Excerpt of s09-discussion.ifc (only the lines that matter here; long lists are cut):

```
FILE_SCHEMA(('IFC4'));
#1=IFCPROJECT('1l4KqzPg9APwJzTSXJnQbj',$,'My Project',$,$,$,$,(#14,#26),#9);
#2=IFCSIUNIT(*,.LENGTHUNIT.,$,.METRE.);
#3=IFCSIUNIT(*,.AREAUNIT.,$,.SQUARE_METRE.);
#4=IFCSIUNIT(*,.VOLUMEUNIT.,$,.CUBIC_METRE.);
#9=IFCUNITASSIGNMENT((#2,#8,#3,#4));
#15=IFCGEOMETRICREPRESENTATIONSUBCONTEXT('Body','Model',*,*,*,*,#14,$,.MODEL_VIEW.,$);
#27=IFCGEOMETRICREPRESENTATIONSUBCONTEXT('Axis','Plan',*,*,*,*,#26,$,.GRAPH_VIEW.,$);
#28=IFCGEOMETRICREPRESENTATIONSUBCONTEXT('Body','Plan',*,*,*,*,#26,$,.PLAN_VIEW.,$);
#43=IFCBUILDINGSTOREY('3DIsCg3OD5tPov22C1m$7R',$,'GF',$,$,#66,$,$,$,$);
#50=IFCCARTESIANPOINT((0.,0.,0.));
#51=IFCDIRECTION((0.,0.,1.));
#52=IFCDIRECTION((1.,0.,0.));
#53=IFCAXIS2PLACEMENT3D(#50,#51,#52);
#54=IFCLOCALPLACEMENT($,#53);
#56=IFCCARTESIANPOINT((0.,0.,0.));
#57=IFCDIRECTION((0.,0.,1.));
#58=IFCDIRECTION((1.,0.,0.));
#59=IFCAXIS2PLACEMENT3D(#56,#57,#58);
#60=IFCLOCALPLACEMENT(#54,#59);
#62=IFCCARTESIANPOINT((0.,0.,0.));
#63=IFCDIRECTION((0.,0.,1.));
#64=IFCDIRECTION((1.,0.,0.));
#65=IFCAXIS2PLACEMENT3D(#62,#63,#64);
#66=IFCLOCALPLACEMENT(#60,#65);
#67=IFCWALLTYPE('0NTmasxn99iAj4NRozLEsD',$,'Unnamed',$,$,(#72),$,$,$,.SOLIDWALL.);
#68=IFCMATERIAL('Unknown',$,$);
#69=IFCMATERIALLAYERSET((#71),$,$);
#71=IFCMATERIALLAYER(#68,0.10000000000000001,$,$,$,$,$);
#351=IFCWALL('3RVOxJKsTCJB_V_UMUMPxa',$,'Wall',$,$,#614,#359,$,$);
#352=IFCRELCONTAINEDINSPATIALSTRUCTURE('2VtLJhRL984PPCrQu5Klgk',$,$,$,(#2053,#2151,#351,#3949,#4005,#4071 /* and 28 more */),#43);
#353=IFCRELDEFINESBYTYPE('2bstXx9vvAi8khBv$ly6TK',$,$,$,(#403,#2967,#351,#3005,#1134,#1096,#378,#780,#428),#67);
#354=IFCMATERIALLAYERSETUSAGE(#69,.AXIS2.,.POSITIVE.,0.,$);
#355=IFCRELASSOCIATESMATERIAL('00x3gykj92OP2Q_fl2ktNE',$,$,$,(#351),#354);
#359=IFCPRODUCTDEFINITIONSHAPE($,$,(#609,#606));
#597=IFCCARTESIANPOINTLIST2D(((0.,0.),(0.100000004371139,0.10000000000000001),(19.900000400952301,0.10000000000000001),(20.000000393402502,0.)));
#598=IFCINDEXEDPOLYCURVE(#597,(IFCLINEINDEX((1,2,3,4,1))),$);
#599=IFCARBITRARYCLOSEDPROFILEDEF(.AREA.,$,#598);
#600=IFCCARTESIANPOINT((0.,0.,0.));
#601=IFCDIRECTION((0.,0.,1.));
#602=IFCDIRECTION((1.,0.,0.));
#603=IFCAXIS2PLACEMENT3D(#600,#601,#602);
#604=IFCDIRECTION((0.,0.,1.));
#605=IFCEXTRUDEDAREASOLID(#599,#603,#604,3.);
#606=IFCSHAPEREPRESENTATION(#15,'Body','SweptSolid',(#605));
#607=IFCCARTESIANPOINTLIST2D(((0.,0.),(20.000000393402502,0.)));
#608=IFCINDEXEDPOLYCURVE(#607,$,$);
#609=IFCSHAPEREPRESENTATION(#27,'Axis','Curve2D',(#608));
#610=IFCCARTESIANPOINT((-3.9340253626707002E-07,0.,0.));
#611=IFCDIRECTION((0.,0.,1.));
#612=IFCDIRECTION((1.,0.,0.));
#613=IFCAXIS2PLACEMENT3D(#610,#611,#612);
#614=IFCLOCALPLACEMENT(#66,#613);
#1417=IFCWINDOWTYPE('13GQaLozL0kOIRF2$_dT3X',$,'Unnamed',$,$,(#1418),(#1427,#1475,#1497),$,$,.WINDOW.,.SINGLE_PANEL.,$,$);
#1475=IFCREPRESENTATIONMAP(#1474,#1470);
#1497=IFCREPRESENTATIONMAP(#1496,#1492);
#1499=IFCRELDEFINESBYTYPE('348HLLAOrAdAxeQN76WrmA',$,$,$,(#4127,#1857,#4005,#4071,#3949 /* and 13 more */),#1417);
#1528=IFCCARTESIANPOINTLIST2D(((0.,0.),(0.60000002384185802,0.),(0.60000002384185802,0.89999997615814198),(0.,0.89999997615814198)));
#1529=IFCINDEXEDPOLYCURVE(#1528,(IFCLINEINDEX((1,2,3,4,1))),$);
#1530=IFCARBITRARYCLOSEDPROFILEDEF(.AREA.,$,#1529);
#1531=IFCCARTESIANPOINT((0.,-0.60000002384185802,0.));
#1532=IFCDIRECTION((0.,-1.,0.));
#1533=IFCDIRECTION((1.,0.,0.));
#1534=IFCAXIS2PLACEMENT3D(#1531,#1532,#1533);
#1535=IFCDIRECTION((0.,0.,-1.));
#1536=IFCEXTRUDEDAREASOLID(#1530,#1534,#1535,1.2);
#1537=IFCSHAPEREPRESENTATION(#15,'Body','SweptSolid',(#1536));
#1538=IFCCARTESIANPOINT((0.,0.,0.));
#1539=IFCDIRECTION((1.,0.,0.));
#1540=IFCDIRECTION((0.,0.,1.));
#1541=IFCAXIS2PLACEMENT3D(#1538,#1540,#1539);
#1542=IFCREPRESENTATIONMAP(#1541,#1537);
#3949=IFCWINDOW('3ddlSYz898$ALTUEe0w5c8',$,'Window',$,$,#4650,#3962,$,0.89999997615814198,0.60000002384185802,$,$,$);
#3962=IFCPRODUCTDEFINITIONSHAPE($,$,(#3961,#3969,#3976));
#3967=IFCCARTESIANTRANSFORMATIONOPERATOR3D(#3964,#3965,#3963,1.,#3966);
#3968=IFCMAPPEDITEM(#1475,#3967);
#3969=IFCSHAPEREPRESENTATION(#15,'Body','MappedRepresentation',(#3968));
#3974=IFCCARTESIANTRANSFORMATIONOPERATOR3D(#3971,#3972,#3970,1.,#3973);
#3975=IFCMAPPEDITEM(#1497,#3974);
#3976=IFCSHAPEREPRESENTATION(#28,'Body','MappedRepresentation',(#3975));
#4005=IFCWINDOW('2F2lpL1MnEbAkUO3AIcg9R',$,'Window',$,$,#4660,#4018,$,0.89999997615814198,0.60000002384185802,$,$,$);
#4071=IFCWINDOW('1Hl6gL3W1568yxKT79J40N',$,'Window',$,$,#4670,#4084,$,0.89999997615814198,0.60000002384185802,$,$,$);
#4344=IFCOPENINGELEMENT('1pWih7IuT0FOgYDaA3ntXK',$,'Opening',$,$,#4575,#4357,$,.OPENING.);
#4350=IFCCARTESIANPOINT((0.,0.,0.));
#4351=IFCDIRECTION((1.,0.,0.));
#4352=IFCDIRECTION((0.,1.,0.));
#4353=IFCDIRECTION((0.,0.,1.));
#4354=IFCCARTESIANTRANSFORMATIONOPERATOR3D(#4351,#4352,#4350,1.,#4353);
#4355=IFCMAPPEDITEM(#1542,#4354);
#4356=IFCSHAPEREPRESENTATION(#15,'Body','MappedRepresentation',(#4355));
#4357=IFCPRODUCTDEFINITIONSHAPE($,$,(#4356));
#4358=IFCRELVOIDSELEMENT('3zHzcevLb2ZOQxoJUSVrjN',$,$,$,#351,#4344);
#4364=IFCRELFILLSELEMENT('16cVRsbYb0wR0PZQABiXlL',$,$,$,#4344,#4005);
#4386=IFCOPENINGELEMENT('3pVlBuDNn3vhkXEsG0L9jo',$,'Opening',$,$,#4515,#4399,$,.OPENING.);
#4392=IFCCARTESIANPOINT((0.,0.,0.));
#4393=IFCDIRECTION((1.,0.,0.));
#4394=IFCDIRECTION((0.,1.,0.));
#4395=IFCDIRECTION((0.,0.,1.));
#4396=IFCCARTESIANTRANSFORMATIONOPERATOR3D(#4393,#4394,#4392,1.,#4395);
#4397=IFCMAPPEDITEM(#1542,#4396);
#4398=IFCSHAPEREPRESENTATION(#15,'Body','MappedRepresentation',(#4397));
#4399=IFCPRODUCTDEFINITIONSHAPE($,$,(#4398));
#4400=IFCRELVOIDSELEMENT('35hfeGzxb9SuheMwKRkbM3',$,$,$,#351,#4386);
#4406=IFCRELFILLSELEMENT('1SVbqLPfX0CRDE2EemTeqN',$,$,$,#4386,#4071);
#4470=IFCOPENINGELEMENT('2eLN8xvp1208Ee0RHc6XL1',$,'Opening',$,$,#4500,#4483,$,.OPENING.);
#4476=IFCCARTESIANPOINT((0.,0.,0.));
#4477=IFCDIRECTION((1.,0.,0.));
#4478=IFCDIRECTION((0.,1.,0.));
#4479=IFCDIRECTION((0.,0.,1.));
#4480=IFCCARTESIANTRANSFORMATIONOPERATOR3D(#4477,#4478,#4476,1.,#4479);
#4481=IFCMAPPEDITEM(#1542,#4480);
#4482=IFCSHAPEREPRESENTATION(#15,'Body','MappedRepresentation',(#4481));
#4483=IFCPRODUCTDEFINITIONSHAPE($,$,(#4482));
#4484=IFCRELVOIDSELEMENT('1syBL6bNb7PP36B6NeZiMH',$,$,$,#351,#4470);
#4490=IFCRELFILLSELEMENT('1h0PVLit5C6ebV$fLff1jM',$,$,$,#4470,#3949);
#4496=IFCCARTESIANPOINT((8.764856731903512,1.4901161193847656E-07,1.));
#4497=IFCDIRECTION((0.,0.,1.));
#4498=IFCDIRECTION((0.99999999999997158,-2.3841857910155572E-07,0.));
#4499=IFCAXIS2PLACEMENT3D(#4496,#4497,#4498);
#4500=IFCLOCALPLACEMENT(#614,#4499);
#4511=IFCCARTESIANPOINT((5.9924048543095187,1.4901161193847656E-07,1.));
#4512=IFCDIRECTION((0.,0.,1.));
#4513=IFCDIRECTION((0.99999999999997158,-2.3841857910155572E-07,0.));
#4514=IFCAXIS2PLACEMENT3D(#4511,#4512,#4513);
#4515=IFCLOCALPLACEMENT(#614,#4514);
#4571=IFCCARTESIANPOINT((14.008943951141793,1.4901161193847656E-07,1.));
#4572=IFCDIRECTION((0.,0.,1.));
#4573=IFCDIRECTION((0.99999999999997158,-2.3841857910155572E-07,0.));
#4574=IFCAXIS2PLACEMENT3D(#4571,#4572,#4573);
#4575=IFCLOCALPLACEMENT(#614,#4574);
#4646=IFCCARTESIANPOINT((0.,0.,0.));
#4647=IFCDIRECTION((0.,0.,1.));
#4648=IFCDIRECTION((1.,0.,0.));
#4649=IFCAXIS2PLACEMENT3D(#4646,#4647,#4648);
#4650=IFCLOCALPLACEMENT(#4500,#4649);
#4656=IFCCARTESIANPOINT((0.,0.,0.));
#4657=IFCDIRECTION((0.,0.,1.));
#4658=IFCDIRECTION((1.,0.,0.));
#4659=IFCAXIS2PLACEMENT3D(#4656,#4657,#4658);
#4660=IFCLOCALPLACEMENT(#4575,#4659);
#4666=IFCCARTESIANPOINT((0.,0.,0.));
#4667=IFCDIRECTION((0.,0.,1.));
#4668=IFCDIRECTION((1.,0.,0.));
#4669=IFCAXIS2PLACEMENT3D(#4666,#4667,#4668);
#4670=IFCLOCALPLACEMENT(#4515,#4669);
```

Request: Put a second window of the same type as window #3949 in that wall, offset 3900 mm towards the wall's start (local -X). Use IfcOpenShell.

```python
import ifcopenshell
import ifcopenshell.api.feature
import ifcopenshell.api.geometry
import ifcopenshell.api.root
import ifcopenshell.geom
import ifcopenshell.util.element
import ifcopenshell.util.placement
import ifcopenshell.util.shape
import ifcopenshell.util.unit

model = ifcopenshell.open("s09-discussion.ifc")
unit_scale = ifcopenshell.util.unit.calculate_unit_scale(model)
settings = ifcopenshell.geom.settings()


def volume(element):
    """Net volume in cubic metres, openings subtracted."""
    shape = ifcopenshell.geom.create_shape(settings, element)
    return ifcopenshell.util.shape.get_volume(shape.geometry)


window = model.by_id(3949)
opening = window.FillsVoids[0].RelatingOpeningElement
wall = opening.VoidsElements[0].RelatingBuildingElement
before = volume(wall)
shift = ifcopenshell.util.placement.get_local_placement(wall.ObjectPlacement)[:3, 0] * -3.9 / unit_scale

# copy_class copies the void relationship, type, container and properties, but no geometry.
new_opening = ifcopenshell.api.root.copy_class(model, product=opening)
new_opening.Representation = ifcopenshell.util.element.copy_deep(
    model, opening.Representation, exclude=["IfcGeometricRepresentationContext", "IfcRepresentationMap"]
)
new_window = ifcopenshell.api.root.copy_class(model, product=window)
new_window.Representation = ifcopenshell.util.element.copy_deep(
    model, window.Representation, exclude=["IfcGeometricRepresentationContext", "IfcRepresentationMap"]
)
ifcopenshell.api.feature.add_filling(model, opening=new_opening, element=new_window)

for old, new in ((opening, new_opening), (window, new_window)):
    matrix = ifcopenshell.util.placement.get_local_placement(old.ObjectPlacement)
    matrix[:3, 3] += shift
    ifcopenshell.api.geometry.edit_object_placement(model, product=new, matrix=matrix, is_si=False)

after = volume(wall)

print(f"wall volume {before:.3f} -> {after:.3f} m3")

model.write("s09-discussion_v2.ifc")
```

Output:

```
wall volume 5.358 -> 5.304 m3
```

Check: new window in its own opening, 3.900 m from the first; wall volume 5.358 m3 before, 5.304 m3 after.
